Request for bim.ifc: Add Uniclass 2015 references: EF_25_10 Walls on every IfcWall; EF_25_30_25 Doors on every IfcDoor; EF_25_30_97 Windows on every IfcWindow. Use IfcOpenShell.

First a look at what the model holds.

```python
import ifcopenshell

model = ifcopenshell.open("bim.ifc")
print(model.schema)
print("classifications:", [c.Name for c in model.by_type("IfcClassification")])
for ifc_class in ("IfcDoor", "IfcRoof", "IfcStair", "IfcWall", "IfcWindow"):
    print(ifc_class, len(model.by_type(ifc_class)))
```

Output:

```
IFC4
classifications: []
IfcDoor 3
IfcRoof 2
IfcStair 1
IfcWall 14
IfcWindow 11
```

```python
import ifcopenshell
import ifcopenshell.api.classification

model = ifcopenshell.open("bim.ifc")

system = ifcopenshell.api.classification.add_classification(model, classification="Uniclass 2015")

codes = {
    "IfcWall": ("EF_25_10", "Walls"),
    "IfcDoor": ("EF_25_30_25", "Doors"),
    "IfcWindow": ("EF_25_30_97", "Windows"),
}
for ifc_class, (code, name) in codes.items():
    products = model.by_type(ifc_class)
    ifcopenshell.api.classification.add_reference(
        model, products=products, classification=system, identification=code, name=name
    )
    print(code, len(products))

model.write("bim-out.ifc")
```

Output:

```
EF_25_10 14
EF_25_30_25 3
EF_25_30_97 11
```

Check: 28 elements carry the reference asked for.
